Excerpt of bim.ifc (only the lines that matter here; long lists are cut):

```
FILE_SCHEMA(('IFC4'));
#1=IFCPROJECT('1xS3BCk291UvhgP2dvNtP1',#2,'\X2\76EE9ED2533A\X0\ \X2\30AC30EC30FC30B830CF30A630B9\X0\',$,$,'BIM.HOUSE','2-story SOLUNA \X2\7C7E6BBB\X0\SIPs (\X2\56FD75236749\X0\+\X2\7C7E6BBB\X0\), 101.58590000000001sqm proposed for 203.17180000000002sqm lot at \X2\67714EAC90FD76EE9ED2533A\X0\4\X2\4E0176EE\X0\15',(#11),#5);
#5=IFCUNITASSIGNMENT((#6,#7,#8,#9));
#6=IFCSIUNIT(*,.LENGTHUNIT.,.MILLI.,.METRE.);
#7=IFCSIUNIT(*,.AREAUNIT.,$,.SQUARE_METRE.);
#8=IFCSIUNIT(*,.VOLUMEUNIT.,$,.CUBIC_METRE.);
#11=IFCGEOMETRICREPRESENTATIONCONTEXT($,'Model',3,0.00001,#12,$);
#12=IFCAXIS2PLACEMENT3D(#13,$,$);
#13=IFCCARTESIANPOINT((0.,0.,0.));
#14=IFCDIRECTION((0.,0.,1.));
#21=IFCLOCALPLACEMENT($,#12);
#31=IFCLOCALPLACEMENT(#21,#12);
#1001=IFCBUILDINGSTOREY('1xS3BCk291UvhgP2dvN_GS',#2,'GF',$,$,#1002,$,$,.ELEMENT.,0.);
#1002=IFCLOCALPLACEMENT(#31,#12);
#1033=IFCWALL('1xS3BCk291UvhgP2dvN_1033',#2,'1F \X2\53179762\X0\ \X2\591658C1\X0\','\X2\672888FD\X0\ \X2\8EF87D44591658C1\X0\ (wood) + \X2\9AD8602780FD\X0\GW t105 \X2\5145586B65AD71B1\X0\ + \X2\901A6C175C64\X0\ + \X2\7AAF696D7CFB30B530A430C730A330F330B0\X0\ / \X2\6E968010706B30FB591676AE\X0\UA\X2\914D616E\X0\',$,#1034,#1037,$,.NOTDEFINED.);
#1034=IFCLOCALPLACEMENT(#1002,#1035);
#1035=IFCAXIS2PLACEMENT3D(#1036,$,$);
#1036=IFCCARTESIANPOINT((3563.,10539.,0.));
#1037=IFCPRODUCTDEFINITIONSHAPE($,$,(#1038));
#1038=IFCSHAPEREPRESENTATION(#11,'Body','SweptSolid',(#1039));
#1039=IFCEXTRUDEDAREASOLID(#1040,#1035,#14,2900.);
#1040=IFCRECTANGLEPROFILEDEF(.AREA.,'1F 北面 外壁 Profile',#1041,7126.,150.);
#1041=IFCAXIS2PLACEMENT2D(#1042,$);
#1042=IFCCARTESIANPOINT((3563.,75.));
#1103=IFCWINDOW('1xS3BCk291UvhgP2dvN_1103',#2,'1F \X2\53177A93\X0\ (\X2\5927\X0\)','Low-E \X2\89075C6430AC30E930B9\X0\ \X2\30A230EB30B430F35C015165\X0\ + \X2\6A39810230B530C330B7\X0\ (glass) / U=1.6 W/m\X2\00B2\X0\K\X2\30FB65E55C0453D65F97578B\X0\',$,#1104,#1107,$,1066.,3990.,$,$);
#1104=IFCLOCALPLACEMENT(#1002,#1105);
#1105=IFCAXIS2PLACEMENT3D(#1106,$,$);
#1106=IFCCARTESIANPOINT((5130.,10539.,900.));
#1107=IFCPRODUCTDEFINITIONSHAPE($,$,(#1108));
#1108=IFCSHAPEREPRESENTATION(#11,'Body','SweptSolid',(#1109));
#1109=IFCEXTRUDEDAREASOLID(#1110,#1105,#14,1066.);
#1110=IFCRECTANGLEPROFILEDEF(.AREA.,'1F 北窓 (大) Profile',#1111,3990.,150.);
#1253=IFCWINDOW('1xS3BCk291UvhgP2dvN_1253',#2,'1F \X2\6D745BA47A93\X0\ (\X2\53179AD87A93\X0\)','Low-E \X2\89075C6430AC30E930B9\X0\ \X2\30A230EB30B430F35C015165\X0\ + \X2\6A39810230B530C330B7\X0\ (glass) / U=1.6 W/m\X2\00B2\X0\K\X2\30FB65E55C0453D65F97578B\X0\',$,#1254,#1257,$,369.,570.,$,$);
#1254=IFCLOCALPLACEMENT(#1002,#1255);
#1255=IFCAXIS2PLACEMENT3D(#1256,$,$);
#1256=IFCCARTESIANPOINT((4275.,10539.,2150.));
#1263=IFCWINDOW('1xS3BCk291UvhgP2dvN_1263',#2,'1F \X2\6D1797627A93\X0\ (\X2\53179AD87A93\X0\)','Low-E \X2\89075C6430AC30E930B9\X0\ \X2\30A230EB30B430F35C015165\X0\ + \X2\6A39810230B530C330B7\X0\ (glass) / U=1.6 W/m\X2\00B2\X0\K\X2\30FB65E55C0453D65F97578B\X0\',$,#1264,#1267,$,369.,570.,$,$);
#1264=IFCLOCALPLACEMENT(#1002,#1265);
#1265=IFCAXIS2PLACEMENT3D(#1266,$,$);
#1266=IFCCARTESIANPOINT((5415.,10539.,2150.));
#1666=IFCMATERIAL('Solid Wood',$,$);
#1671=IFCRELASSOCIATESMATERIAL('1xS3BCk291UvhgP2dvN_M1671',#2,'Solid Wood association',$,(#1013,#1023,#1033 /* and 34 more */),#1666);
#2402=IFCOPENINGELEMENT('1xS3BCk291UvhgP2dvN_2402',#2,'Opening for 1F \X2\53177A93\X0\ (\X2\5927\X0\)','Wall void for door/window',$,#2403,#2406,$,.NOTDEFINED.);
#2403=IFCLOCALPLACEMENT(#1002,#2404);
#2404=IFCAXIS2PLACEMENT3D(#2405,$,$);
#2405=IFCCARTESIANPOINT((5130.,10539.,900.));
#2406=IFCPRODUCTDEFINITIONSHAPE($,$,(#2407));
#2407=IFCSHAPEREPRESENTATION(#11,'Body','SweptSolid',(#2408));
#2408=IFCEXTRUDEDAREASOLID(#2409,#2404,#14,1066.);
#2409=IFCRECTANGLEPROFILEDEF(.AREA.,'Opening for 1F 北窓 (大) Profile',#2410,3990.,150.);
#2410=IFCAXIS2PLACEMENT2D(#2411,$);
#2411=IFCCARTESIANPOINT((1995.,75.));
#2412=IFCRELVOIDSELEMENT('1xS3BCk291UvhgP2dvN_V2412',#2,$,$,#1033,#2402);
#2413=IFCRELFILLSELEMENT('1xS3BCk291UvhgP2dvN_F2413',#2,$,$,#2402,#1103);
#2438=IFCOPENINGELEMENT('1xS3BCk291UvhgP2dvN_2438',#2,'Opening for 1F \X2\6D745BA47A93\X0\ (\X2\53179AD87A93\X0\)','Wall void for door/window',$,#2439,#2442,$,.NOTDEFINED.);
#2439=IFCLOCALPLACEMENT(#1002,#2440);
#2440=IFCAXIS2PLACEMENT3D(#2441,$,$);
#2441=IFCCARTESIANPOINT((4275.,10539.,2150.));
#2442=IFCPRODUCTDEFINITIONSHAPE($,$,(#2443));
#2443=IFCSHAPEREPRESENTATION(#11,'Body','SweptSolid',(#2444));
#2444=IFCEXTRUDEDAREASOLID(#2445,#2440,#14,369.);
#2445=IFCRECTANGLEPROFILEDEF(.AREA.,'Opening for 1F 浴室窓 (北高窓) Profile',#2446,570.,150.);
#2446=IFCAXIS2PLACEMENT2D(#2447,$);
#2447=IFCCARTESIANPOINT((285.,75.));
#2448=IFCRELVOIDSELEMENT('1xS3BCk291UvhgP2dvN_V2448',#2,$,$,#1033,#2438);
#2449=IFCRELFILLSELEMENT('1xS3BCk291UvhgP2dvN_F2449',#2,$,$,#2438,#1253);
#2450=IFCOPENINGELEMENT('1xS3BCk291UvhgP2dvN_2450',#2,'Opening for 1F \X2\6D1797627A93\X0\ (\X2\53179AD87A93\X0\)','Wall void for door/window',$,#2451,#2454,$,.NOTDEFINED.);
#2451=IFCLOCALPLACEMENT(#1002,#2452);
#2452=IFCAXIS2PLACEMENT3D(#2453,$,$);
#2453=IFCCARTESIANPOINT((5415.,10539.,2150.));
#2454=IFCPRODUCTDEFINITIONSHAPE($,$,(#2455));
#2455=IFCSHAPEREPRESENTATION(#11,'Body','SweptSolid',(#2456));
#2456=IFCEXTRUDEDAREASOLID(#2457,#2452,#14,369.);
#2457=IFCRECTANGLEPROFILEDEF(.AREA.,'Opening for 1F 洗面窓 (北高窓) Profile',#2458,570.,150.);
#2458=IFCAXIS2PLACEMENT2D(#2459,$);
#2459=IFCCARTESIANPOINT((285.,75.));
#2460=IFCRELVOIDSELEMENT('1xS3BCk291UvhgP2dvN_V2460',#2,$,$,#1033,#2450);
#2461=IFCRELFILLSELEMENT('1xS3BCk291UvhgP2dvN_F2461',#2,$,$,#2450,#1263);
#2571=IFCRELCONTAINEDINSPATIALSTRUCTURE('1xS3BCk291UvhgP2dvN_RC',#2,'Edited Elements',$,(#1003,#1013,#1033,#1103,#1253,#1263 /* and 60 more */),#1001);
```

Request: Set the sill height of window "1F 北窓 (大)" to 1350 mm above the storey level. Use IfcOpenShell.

```python
import numpy as np
import ifcopenshell
import ifcopenshell.api.geometry
import ifcopenshell.geom
import ifcopenshell.util.element
import ifcopenshell.util.placement
import ifcopenshell.util.shape
import ifcopenshell.util.unit

model = ifcopenshell.open("bim.ifc")
unit_scale = ifcopenshell.util.unit.calculate_unit_scale(model)

window = model.by_guid("1xS3BCk291UvhgP2dvN_1103")
opening = window.FillsVoids[0].RelatingOpeningElement
storey = ifcopenshell.util.element.get_container(window, ifc_class="IfcBuildingStorey")
level = ifcopenshell.util.placement.get_local_placement(storey.ObjectPlacement)[2, 3]

# The opening's origin need not be at the sill, so measure its lowest point.
shape = ifcopenshell.geom.create_shape(ifcopenshell.geom.settings(), opening)
bottom = ifcopenshell.util.shape.get_shape_bottom_elevation(shape, shape.geometry) / unit_scale
dz = level + 1.35 / unit_scale - bottom

shift = np.array([0.0, 0.0, dz])
# The window is not placed relative to its opening, so move both.
for product in (opening, window):
    matrix = ifcopenshell.util.placement.get_local_placement(product.ObjectPlacement)
    matrix[:3, 3] += shift
    ifcopenshell.api.geometry.edit_object_placement(model, product=product, matrix=matrix, is_si=False)

print(f"moved by {dz * unit_scale:+.3f} m")

model.write("bim_updated.ifc")
```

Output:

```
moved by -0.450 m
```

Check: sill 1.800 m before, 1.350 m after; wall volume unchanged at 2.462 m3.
